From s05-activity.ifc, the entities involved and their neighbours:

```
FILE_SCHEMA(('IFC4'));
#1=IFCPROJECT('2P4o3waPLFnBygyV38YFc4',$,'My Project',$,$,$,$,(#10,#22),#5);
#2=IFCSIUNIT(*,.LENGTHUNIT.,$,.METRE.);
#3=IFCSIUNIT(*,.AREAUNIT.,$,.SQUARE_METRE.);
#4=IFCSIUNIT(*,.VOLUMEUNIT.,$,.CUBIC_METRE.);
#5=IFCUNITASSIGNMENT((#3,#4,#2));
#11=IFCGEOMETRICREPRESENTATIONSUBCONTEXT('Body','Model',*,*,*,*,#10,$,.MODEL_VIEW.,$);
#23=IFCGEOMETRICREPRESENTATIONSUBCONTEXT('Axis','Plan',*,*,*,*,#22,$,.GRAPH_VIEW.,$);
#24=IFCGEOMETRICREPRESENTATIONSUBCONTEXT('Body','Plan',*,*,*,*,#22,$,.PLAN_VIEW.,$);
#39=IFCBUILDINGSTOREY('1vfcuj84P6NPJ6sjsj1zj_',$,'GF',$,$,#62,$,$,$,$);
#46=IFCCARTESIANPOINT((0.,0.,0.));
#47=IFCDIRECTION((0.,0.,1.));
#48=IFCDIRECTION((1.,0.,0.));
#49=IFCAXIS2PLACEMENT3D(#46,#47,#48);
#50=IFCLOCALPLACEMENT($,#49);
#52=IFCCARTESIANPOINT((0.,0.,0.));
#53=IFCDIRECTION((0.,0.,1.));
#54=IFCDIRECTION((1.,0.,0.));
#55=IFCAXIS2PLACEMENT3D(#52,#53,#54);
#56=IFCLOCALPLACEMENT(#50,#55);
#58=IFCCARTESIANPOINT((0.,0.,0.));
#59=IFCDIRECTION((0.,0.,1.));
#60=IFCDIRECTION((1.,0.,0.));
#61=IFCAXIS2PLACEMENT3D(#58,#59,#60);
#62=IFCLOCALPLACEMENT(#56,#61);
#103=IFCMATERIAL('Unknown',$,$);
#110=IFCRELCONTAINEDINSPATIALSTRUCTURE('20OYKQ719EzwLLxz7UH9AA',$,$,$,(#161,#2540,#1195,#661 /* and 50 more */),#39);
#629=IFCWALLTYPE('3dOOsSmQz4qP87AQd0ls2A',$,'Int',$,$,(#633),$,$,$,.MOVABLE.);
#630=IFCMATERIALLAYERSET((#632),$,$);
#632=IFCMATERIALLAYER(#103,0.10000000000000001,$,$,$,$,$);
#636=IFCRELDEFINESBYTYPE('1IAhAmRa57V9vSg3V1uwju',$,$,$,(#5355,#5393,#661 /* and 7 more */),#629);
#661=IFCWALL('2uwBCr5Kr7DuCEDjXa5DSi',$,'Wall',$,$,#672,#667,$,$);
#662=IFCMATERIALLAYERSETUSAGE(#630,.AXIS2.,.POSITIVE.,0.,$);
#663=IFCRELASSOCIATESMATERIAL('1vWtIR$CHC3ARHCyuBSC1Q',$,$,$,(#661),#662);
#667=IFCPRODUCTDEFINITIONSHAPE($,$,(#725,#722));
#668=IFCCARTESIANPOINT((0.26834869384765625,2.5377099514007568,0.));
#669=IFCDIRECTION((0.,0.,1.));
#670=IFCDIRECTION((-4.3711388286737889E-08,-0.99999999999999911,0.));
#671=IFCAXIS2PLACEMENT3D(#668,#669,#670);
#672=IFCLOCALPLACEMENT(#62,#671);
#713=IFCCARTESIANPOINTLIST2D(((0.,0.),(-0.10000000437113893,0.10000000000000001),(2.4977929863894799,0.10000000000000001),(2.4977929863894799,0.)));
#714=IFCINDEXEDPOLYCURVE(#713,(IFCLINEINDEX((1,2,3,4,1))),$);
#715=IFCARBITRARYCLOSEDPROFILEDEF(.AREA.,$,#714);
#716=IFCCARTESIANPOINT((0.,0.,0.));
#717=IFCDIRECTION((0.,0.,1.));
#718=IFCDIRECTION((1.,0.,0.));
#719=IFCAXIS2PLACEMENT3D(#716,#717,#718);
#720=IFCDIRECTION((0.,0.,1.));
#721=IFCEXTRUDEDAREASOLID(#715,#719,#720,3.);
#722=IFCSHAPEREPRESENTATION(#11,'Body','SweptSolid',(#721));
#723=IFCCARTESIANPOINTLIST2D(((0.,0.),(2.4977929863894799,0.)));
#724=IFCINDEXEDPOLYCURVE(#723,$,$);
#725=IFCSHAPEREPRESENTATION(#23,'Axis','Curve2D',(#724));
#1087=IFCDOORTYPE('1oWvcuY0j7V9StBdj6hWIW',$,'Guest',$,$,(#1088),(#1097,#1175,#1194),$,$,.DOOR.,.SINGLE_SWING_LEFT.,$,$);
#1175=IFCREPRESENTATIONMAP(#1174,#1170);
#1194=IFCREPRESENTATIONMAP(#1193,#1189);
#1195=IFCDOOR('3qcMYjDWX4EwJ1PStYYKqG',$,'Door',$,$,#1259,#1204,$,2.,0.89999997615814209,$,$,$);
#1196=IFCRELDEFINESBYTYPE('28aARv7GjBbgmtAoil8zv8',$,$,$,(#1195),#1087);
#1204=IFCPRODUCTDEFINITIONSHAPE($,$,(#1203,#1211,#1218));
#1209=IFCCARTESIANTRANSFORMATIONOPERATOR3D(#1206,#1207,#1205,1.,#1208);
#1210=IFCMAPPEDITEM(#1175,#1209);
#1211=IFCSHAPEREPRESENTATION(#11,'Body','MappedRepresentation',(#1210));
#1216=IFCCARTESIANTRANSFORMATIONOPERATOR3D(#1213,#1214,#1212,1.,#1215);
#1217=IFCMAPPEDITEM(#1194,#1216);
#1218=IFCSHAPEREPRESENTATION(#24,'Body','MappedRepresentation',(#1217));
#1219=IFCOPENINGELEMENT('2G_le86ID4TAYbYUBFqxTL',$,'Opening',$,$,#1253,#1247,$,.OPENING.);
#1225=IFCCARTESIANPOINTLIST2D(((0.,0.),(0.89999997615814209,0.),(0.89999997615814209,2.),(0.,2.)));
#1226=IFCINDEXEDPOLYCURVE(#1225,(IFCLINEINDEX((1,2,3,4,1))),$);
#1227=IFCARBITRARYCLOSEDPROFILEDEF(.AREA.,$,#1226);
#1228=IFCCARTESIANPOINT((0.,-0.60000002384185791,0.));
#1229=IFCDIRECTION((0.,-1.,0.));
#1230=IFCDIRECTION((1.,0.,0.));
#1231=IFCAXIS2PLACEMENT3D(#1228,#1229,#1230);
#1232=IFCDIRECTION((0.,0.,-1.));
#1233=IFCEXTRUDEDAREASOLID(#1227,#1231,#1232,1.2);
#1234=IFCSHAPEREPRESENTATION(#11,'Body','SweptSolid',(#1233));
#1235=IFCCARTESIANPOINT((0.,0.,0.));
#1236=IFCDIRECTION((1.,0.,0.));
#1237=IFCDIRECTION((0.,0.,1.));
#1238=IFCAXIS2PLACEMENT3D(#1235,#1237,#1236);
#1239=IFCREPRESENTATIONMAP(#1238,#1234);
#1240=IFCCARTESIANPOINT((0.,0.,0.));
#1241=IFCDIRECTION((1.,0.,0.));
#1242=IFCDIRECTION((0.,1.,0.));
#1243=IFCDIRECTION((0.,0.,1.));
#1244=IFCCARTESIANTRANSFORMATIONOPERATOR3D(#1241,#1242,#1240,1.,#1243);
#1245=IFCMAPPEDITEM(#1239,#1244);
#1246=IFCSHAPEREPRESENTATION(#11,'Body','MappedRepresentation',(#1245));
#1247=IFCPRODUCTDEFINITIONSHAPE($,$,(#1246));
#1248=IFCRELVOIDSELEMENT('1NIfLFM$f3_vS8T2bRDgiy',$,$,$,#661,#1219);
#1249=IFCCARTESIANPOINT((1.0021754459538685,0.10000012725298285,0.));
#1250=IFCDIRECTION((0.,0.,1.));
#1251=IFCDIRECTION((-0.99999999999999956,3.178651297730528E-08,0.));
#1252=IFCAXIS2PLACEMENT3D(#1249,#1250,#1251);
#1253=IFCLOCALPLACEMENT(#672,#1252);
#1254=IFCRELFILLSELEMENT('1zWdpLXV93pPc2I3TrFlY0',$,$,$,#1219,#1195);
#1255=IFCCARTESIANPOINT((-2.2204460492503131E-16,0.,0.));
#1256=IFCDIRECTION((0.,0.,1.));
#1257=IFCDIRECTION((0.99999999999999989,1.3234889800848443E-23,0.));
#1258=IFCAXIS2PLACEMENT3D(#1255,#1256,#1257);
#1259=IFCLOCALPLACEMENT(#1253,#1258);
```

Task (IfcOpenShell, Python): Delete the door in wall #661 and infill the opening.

```python
import ifcopenshell
import ifcopenshell.api.feature
import ifcopenshell.api.root
import ifcopenshell.geom
import ifcopenshell.util.shape

model = ifcopenshell.open("s05-activity.ifc")
settings = ifcopenshell.geom.settings()


def volume(element):
    """Net volume in cubic metres, openings subtracted."""
    shape = ifcopenshell.geom.create_shape(settings, element)
    return ifcopenshell.util.shape.get_volume(shape.geometry)


door = model.by_guid("3qcMYjDWX4EwJ1PStYYKqG")
opening = door.FillsVoids[0].RelatingOpeningElement
wall = opening.VoidsElements[0].RelatingBuildingElement
before = volume(wall)

ifcopenshell.api.root.remove_product(model, product=door)
ifcopenshell.api.feature.remove_feature(model, feature=opening)

after = volume(wall)

print(f"wall volume {before:.3f} -> {after:.3f} m3")

model.write("s05-activity-out.ifc")
```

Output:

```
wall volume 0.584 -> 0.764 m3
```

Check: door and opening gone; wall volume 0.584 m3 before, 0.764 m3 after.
